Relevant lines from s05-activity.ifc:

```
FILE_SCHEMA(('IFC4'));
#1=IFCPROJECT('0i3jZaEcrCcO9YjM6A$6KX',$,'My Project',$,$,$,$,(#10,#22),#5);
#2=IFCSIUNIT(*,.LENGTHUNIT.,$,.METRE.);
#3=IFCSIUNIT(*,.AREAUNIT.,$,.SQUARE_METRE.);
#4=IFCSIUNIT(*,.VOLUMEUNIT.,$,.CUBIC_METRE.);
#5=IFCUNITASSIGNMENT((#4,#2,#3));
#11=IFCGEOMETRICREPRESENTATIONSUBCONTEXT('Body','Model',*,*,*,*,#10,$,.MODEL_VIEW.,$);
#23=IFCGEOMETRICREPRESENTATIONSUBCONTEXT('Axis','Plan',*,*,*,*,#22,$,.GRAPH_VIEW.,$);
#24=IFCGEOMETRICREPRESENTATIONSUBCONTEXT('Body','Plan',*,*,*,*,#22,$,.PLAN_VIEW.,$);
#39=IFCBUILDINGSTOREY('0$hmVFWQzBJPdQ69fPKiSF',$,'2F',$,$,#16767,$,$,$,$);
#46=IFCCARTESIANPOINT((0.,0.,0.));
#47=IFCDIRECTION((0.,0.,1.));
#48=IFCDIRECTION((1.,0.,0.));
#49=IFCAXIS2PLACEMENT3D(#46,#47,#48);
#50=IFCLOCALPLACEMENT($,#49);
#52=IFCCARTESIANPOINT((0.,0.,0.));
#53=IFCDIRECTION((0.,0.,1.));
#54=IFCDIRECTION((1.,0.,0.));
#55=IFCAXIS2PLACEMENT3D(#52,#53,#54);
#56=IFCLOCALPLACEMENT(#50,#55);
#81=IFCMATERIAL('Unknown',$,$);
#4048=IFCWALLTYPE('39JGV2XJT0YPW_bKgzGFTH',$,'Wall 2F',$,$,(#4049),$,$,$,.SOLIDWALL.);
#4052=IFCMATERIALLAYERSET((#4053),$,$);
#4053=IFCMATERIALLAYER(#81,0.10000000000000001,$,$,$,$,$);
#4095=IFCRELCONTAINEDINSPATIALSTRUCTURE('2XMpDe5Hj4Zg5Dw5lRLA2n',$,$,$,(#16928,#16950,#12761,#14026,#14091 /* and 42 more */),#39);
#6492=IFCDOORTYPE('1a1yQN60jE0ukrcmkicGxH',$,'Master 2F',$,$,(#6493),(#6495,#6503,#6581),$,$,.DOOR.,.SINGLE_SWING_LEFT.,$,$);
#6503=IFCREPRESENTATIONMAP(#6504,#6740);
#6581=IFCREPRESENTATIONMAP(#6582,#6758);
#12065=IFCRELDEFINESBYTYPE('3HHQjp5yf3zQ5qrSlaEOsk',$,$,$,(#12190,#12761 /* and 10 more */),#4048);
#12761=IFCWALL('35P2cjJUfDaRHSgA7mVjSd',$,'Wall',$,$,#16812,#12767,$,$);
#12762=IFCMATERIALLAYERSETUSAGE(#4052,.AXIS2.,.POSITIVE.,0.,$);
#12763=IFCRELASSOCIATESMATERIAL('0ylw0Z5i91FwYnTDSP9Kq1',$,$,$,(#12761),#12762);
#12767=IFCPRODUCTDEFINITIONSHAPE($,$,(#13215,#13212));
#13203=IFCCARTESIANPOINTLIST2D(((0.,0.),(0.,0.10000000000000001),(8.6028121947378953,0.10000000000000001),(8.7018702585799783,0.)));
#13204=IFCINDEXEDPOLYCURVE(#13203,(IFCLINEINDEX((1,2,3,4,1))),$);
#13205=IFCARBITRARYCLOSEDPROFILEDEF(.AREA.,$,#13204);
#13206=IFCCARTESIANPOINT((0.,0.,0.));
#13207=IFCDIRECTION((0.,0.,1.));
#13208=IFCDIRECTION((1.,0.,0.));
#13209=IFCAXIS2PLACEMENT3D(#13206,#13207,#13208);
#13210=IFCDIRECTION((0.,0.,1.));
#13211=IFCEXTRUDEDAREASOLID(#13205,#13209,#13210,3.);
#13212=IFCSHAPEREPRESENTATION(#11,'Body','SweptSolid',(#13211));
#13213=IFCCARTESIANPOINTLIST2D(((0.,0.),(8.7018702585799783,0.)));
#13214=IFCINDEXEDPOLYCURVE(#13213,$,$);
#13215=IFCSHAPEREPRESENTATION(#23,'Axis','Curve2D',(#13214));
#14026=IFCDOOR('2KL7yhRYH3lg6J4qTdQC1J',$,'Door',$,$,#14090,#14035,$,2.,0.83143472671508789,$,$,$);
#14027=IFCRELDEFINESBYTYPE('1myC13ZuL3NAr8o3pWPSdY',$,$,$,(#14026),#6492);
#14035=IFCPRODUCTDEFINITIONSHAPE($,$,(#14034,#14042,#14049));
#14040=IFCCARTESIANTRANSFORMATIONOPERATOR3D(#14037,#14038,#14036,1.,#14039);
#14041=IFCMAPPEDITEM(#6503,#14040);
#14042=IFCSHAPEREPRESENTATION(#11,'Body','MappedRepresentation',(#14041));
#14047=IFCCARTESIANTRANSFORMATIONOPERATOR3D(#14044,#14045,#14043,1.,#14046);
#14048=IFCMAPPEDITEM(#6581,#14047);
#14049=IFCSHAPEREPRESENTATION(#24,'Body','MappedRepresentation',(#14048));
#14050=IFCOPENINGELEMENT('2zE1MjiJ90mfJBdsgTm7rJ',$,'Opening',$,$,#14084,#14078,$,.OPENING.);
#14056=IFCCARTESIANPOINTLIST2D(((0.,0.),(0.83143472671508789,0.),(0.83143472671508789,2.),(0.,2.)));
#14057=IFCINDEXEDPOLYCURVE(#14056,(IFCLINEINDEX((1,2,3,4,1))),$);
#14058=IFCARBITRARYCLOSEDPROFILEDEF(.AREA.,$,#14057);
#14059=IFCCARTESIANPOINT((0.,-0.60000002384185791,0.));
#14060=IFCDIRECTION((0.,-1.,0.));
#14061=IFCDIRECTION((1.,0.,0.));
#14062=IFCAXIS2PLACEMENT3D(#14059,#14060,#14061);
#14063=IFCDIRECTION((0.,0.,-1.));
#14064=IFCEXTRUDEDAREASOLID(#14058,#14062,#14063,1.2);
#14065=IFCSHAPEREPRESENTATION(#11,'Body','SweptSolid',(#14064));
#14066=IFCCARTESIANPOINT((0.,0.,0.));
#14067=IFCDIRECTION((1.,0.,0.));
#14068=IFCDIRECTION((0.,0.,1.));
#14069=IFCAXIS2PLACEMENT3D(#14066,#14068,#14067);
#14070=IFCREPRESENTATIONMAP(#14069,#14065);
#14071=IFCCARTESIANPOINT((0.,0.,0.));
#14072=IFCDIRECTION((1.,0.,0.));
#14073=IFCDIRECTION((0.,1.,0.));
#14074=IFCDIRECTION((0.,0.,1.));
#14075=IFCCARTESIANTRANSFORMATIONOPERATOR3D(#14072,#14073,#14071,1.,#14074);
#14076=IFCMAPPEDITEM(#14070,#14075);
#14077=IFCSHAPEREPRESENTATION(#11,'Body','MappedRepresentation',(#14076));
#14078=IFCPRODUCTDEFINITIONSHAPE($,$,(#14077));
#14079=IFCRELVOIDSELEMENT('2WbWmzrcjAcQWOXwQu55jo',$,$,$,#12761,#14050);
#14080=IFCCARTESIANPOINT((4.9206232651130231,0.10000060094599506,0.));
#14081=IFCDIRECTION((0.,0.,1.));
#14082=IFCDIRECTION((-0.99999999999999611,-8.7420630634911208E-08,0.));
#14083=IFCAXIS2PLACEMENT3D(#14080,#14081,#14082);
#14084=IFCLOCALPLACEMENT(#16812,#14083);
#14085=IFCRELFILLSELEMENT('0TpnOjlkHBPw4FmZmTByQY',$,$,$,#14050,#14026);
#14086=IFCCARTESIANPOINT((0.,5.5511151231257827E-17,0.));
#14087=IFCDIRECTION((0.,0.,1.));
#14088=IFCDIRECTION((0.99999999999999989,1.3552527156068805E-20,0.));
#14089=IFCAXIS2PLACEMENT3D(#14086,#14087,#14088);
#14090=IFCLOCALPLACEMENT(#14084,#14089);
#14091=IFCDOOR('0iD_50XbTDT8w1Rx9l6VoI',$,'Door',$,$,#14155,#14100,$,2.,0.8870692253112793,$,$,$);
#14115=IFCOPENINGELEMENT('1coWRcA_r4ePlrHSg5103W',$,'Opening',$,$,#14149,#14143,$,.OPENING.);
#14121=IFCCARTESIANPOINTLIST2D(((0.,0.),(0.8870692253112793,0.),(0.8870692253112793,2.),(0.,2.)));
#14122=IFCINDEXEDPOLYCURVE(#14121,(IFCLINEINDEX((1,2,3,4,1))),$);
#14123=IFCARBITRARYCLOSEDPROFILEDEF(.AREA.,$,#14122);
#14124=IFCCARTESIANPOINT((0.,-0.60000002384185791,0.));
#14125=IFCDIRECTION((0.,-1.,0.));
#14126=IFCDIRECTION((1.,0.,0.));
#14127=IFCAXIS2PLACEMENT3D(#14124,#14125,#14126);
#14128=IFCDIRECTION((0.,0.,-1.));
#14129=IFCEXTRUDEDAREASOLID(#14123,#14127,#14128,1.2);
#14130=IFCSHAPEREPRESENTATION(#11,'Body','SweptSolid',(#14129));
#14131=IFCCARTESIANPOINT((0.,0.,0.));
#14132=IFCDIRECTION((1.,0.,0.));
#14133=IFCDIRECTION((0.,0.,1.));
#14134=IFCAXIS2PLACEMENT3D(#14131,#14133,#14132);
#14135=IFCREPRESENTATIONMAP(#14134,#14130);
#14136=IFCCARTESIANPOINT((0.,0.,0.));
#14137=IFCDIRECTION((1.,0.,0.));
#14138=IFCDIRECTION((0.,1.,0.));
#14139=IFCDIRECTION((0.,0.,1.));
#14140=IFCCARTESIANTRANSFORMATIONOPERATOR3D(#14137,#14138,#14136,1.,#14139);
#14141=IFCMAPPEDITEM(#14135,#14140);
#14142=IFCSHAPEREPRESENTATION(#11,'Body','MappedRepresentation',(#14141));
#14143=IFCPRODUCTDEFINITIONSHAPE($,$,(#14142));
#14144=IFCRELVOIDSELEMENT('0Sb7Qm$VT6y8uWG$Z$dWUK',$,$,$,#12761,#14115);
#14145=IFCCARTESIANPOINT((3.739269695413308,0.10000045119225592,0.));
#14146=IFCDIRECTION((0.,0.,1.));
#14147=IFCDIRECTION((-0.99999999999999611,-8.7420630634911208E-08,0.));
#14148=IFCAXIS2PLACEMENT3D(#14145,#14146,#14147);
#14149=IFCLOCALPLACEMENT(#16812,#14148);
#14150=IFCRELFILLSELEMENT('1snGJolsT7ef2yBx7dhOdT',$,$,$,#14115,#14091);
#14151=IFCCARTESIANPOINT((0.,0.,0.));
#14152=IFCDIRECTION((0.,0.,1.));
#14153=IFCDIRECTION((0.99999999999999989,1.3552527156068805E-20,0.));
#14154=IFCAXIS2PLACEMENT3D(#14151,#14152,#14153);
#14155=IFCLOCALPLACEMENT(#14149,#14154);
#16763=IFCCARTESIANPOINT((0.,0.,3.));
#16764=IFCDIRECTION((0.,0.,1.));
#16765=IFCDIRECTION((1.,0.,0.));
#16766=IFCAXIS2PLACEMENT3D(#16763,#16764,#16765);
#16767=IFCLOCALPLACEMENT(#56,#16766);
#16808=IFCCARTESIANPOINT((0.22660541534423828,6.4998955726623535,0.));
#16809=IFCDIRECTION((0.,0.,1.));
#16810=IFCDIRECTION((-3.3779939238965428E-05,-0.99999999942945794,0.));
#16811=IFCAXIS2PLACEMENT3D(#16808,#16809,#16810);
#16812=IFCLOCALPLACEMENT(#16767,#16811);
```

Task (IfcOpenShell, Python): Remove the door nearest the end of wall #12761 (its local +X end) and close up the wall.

```python
import ifcopenshell
import ifcopenshell.api.feature
import ifcopenshell.api.root
import ifcopenshell.geom
import ifcopenshell.util.shape

model = ifcopenshell.open("s05-activity.ifc")
settings = ifcopenshell.geom.settings()


def volume(element):
    """Net volume in cubic metres, openings subtracted."""
    shape = ifcopenshell.geom.create_shape(settings, element)
    return ifcopenshell.util.shape.get_volume(shape.geometry)


door = model.by_guid("2KL7yhRYH3lg6J4qTdQC1J")
opening = door.FillsVoids[0].RelatingOpeningElement
wall = opening.VoidsElements[0].RelatingBuildingElement
before = volume(wall)

ifcopenshell.api.root.remove_product(model, product=door)
ifcopenshell.api.feature.remove_feature(model, feature=opening)

after = volume(wall)

print(f"wall volume {before:.3f} -> {after:.3f} m3")

model.write("s05-activity_edited.ifc")
```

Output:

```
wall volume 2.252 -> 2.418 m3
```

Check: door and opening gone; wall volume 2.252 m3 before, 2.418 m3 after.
